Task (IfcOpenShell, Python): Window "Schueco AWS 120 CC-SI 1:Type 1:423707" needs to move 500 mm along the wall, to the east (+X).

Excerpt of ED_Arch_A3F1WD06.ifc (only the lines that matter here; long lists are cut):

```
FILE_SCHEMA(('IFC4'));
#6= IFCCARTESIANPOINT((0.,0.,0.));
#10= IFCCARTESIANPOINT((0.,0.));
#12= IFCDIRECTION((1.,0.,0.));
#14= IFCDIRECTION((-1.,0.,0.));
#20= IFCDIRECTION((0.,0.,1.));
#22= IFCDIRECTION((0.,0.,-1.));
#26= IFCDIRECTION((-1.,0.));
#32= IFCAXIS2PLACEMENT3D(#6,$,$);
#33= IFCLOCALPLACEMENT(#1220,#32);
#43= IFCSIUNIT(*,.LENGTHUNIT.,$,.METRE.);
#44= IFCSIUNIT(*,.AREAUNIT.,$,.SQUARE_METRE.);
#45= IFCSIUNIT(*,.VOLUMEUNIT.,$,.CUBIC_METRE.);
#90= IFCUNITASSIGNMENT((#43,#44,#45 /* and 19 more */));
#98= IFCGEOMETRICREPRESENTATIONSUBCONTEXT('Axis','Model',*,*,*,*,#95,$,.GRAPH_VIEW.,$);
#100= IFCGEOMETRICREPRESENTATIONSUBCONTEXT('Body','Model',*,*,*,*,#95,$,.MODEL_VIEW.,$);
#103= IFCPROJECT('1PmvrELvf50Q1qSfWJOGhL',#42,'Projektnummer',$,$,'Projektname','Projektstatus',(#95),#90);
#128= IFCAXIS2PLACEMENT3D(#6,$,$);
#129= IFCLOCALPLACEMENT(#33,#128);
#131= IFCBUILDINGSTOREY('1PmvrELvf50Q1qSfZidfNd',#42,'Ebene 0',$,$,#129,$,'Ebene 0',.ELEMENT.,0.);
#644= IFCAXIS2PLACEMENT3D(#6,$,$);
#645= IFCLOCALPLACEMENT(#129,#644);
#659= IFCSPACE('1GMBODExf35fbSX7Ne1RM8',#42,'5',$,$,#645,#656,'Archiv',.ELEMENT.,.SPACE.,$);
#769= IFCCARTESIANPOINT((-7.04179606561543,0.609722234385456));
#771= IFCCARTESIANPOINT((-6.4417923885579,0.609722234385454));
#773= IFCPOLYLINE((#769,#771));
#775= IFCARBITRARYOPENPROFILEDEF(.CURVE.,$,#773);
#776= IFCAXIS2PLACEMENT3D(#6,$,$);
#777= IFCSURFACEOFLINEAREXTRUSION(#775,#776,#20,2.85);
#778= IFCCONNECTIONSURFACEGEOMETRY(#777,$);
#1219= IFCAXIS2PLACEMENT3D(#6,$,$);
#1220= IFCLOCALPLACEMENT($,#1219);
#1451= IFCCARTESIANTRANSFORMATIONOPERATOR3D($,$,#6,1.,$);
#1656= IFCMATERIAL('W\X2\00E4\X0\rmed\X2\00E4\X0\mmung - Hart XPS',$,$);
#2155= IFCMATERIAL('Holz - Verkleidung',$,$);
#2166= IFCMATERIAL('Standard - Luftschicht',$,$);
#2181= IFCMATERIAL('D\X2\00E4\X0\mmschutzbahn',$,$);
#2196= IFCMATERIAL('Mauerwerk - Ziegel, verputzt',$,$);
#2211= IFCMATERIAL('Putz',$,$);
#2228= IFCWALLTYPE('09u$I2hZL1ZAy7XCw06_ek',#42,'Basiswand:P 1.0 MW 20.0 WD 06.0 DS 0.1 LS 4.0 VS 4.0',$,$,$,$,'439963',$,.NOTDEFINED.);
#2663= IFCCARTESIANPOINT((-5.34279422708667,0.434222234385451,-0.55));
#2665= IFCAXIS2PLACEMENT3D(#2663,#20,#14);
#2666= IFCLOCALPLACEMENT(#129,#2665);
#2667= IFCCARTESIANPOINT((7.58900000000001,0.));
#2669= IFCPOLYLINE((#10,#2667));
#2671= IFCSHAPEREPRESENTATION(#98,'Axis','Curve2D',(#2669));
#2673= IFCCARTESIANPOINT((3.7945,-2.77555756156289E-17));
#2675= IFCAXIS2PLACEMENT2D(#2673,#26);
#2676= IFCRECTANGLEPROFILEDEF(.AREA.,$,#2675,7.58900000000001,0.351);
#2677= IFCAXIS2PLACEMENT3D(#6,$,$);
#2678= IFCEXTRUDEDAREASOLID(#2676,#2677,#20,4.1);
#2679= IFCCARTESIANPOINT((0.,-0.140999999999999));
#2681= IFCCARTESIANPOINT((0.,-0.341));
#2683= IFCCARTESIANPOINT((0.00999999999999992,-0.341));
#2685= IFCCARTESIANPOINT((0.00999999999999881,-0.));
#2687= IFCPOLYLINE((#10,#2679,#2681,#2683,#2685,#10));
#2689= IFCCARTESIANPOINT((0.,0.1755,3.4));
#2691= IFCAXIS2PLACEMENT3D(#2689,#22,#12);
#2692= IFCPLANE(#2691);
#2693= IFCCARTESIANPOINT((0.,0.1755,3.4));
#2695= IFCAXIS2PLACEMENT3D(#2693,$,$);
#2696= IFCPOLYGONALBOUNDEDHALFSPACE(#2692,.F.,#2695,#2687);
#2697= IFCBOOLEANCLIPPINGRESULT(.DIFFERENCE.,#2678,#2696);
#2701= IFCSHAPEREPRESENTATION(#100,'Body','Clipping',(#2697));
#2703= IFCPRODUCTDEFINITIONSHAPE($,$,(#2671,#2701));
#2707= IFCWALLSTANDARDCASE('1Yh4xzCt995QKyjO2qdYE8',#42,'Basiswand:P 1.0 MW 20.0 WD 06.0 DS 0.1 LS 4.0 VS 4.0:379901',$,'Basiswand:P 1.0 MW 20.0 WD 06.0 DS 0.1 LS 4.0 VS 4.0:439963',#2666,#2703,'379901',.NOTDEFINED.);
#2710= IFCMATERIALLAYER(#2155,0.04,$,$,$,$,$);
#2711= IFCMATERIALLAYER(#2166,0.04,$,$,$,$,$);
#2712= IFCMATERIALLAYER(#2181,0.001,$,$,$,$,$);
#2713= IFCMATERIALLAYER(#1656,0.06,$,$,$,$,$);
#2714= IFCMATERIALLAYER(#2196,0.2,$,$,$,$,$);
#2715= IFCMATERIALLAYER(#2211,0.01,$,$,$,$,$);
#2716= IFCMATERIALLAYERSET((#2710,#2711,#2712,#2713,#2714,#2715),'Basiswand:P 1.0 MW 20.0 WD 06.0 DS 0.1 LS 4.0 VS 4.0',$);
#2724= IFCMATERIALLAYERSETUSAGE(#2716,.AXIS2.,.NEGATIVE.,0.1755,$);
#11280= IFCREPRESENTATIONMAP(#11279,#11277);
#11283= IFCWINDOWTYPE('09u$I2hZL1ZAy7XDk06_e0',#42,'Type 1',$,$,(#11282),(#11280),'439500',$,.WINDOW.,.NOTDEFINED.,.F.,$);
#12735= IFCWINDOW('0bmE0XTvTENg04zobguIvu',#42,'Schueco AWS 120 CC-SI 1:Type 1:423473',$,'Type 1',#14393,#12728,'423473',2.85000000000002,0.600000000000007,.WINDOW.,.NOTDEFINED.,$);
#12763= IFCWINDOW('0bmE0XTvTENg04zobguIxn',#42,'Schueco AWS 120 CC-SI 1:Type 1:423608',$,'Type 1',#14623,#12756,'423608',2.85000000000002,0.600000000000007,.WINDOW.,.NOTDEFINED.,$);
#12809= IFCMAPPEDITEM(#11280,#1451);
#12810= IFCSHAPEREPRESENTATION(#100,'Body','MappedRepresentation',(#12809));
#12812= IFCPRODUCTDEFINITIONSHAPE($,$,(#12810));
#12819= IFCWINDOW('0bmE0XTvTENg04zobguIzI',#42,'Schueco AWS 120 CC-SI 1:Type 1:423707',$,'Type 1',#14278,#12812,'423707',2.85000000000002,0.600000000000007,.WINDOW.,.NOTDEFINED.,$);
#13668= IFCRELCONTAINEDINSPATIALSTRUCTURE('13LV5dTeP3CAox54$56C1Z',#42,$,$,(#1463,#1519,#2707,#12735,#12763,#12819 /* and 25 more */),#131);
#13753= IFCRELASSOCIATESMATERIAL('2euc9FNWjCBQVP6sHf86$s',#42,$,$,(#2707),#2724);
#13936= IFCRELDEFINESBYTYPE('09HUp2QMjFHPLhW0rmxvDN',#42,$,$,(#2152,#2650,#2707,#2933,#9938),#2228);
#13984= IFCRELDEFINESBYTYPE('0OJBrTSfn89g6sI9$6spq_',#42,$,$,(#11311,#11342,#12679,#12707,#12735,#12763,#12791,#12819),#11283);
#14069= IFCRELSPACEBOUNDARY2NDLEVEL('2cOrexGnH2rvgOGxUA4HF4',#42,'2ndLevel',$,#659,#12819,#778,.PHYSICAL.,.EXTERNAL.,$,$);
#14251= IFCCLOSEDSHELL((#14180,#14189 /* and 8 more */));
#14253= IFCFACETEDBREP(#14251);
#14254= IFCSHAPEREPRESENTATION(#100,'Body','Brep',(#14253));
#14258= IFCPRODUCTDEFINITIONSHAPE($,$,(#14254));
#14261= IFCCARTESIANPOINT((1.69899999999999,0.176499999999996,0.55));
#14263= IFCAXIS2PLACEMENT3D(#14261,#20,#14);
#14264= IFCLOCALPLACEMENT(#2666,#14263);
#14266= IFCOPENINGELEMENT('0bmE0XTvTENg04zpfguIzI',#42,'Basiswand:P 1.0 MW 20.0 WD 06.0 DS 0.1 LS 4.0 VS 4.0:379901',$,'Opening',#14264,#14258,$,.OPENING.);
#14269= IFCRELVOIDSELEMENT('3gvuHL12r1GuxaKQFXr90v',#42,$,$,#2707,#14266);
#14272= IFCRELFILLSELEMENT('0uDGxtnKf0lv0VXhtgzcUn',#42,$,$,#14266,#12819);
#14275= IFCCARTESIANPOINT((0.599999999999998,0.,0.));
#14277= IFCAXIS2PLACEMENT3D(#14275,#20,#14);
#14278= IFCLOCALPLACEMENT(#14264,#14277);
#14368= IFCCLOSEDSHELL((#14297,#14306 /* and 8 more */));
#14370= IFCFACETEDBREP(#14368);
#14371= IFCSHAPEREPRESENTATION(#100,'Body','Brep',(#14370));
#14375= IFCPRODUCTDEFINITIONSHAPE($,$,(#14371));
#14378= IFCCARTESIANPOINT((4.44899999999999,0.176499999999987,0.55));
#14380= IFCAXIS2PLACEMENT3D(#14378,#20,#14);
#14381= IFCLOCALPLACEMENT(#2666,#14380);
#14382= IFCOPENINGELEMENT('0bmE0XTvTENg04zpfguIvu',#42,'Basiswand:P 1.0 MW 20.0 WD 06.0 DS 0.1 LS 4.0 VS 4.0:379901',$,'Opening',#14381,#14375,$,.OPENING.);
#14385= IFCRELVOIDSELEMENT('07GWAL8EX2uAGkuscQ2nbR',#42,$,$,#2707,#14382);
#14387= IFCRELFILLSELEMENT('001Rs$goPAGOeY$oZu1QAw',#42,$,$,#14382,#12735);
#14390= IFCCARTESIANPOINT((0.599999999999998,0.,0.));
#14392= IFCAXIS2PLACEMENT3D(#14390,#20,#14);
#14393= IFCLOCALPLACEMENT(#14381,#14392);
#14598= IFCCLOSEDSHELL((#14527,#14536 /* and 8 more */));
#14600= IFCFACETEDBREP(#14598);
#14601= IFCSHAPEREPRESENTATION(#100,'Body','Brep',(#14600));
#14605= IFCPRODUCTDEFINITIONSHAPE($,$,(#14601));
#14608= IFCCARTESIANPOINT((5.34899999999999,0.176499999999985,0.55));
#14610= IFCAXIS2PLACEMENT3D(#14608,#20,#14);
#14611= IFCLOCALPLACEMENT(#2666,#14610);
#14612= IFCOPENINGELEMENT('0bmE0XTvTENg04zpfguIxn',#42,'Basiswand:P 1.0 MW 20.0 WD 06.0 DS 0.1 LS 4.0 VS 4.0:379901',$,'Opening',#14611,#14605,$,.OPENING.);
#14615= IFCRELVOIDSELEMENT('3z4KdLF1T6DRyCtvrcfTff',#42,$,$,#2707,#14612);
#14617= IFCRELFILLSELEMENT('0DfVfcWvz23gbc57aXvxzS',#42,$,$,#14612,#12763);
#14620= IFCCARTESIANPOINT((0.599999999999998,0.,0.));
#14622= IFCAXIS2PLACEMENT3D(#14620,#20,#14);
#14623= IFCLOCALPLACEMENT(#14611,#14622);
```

```python
import numpy as np
import ifcopenshell
import ifcopenshell.api.geometry
import ifcopenshell.util.placement
import ifcopenshell.util.unit

model = ifcopenshell.open("ED_Arch_A3F1WD06.ifc")
unit_scale = ifcopenshell.util.unit.calculate_unit_scale(model)

window = model.by_guid("0bmE0XTvTENg04zobguIzI")
opening = window.FillsVoids[0].RelatingOpeningElement
wall = opening.VoidsElements[0].RelatingBuildingElement

wall_matrix = ifcopenshell.util.placement.get_local_placement(wall.ObjectPlacement)
shift = wall_matrix[:3, 0] * -0.5 / unit_scale
before = ifcopenshell.util.placement.get_local_placement(window.ObjectPlacement)[:3, 3].copy()

# The window is placed relative to its opening, so it follows when the opening moves.
matrix = ifcopenshell.util.placement.get_local_placement(opening.ObjectPlacement)
matrix[:3, 3] += shift
ifcopenshell.api.geometry.edit_object_placement(
    model, product=opening, matrix=matrix, is_si=False, should_transform_children=True
)

# Space boundary surfaces are stored in each space's coordinates; move them too.
for rel in window.ProvidesBoundaries:
    if not rel.ConnectionGeometry:
        continue
    surface = rel.ConnectionGeometry.SurfaceOnRelatingElement
    space_matrix = ifcopenshell.util.placement.get_local_placement(rel.RelatingSpace.ObjectPlacement)
    point = np.array(surface.Position.Location.Coordinates) + space_matrix[:3, :3].T @ shift
    surface.Position = model.createIfcAxis2Placement3D(
        model.createIfcCartesianPoint(point.tolist()), surface.Position.Axis, surface.Position.RefDirection
    )

after = ifcopenshell.util.placement.get_local_placement(window.ObjectPlacement)[:3, 3]
print("window moved by", (after - before).round(3) + 0.0)

model.write("ED_Arch_A3F1WD06_edited.ifc")
```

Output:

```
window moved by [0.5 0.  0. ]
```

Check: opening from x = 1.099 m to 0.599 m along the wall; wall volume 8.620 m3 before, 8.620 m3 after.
